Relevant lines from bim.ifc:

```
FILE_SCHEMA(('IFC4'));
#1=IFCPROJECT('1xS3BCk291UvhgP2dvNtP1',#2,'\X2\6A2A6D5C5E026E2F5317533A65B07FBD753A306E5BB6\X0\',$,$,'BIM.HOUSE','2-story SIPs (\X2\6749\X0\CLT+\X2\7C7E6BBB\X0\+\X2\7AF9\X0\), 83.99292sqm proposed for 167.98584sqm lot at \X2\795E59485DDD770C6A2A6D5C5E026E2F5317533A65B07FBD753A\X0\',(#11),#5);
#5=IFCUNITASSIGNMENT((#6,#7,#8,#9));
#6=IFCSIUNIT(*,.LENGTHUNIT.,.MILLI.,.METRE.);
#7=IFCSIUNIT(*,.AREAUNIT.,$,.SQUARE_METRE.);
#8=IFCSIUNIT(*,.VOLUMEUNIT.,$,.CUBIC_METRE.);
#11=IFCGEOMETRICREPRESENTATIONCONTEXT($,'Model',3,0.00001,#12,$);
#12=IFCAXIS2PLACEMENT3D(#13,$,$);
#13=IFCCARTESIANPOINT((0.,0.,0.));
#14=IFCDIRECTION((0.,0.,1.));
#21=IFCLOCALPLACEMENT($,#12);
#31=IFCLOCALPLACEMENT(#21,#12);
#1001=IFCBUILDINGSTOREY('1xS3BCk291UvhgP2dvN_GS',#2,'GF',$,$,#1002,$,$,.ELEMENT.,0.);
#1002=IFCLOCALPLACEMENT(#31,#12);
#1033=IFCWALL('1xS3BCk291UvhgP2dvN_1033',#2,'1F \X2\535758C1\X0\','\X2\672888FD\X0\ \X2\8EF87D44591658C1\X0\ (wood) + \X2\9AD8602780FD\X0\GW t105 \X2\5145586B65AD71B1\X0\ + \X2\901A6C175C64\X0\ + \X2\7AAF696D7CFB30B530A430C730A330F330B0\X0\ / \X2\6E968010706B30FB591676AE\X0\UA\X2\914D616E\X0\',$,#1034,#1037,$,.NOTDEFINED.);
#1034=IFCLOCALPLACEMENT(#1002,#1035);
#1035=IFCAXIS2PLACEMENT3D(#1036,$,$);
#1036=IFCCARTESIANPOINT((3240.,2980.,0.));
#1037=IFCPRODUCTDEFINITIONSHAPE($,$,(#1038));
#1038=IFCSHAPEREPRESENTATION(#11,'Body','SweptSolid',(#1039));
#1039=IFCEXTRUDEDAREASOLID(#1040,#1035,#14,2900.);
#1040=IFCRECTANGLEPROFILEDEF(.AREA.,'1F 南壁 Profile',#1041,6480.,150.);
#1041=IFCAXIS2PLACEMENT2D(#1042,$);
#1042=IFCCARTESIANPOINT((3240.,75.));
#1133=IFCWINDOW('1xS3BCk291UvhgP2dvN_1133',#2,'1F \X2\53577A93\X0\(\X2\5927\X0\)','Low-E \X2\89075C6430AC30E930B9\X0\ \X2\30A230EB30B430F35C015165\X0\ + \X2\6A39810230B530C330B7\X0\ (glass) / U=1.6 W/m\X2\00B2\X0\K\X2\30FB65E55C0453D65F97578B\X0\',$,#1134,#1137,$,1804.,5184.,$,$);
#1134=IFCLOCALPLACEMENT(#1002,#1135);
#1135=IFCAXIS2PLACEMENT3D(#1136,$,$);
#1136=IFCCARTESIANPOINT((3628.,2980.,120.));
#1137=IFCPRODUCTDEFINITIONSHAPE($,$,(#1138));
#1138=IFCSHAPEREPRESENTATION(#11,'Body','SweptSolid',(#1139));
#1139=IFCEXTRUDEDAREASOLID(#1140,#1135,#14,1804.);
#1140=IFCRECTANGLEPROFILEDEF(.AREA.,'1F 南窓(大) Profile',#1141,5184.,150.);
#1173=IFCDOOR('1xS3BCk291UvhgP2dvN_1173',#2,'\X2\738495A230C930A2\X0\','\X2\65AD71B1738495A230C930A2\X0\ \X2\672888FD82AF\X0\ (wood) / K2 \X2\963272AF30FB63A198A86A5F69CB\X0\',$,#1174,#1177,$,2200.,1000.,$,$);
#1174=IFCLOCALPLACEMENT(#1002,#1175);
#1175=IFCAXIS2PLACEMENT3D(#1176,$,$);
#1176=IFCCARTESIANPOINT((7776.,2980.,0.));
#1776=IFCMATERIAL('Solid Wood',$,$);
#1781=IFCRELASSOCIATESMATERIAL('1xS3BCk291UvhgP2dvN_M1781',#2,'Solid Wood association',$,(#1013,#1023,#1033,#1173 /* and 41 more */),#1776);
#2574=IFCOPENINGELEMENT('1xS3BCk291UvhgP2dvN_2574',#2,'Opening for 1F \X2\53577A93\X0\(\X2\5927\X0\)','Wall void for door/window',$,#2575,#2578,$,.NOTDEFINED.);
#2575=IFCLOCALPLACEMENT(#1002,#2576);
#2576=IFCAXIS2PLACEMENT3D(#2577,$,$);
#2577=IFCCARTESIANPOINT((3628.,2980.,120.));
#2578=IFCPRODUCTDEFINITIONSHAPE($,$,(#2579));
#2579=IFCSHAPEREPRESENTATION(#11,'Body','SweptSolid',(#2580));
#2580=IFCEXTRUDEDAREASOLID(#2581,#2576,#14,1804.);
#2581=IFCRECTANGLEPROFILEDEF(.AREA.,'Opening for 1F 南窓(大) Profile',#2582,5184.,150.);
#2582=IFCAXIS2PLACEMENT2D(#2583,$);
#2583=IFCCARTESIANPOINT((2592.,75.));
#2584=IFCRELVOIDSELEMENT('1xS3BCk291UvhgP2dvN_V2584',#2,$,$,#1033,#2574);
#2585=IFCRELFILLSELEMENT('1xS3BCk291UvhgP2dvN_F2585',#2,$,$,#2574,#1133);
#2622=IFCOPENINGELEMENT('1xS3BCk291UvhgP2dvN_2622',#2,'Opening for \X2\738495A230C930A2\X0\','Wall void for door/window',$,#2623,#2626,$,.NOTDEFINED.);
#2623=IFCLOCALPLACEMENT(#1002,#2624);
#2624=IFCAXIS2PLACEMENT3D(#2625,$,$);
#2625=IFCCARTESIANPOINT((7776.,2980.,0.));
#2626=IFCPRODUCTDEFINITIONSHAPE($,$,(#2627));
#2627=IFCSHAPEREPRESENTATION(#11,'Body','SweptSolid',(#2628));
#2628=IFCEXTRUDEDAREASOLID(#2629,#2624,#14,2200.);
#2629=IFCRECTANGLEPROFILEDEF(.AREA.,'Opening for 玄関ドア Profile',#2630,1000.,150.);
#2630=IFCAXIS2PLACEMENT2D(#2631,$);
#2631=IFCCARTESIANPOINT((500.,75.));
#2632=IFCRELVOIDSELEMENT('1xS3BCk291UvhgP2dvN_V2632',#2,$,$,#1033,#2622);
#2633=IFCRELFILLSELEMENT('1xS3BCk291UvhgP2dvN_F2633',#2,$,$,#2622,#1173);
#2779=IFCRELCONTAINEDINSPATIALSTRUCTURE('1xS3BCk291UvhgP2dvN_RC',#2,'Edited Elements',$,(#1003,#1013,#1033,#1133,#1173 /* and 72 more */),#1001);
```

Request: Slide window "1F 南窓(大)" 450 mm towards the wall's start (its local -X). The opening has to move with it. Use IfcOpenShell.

```python
import ifcopenshell
import ifcopenshell.api.geometry
import ifcopenshell.util.placement

model = ifcopenshell.open("bim.ifc")

window = model.by_guid("1xS3BCk291UvhgP2dvN_1133")
opening = window.FillsVoids[0].RelatingOpeningElement
wall = opening.VoidsElements[0].RelatingBuildingElement

wall_matrix = ifcopenshell.util.placement.get_local_placement(wall.ObjectPlacement)
shift = wall_matrix[:3, 0] * -450.0
before = ifcopenshell.util.placement.get_local_placement(window.ObjectPlacement)[:3, 3].copy()

# The window is not placed relative to its opening, so move both.
for product in (opening, window):
    matrix = ifcopenshell.util.placement.get_local_placement(product.ObjectPlacement)
    matrix[:3, 3] += shift
    ifcopenshell.api.geometry.edit_object_placement(model, product=product, matrix=matrix, is_si=False)

after = ifcopenshell.util.placement.get_local_placement(window.ObjectPlacement)[:3, 3]
print("window moved by", (after - before).round(3) + 0.0)

model.write("bim-out.ifc")
```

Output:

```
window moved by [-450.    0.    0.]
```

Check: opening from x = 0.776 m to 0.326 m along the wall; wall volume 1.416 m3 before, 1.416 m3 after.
